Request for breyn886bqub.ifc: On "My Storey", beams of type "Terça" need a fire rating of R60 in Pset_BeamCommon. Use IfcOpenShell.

First a look at what the model holds.

```python
import ifcopenshell
import ifcopenshell.util.element

model = ifcopenshell.open("breyn886bqub.ifc")
print(model.schema)
storey = next(s for s in model.by_type("IfcBuildingStorey") if s.Name == "My Storey")
beams = [e for e in ifcopenshell.util.element.get_decomposition(storey) if e.is_a("IfcBeam")]
seen = {}
for e in beams:
    element_type = ifcopenshell.util.element.get_type(e)
    key = (element_type.Name if element_type != e and element_type else None, ifcopenshell.util.element.get_pset(e, "Pset_BeamCommon", "FireRating"))
    seen[key] = seen.get(key, 0) + 1
for (name, value), count in sorted(seen.items(), key=str):
    print(count, "x", name, "|", value)
```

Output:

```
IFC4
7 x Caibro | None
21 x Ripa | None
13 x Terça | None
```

```python
import ifcopenshell
import ifcopenshell.api.pset
import ifcopenshell.util.element

model = ifcopenshell.open("breyn886bqub.ifc")

storey = next(s for s in model.by_type("IfcBuildingStorey") if s.Name == "My Storey")
beams = [e for e in ifcopenshell.util.element.get_decomposition(storey) if e.is_a("IfcBeam")]

count = 0
for e in beams:
    element_type = ifcopenshell.util.element.get_type(e)
    if element_type in (None, e) or element_type.Name != "Terça":
        continue
    # add_pset returns the element's existing set when there is one.
    pset = ifcopenshell.api.pset.add_pset(model, product=e, name="Pset_BeamCommon")
    ifcopenshell.api.pset.edit_pset(model, pset=pset, properties={"FireRating": "R60"})
    count += 1

print(count, "beams updated")

model.write("breyn886bqub-out.ifc")
```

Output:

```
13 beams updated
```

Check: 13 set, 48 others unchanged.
